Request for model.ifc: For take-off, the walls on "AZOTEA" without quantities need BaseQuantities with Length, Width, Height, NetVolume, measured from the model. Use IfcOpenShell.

First a look at what the model holds.

```python
import ifcopenshell
import ifcopenshell.util.element
import ifcopenshell.util.unit

model = ifcopenshell.open("model.ifc")
print(model.schema)
for unit_type in ("LENGTHUNIT", "AREAUNIT", "VOLUMEUNIT"):
    print(unit_type, ifcopenshell.util.unit.calculate_unit_scale(model, unit_type))
storey = next(s for s in model.by_type("IfcBuildingStorey") if s.Name == "AZOTEA")
walls = [e for e in ifcopenshell.util.element.get_decomposition(storey) if e.is_a("IfcWall")]
for e in sorted(walls, key=lambda e: e.id()):
    print(e.id(), e.is_a(), e.Name, list(ifcopenshell.util.element.get_psets(e, qtos_only=True)), sep=" | ")
```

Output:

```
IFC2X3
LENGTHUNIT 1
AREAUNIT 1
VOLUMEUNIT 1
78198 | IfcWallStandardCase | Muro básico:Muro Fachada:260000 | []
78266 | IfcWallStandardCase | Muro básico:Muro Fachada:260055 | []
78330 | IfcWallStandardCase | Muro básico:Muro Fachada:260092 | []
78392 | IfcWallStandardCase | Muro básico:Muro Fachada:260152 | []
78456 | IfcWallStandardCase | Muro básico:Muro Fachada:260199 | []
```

```python
import ifcopenshell
import ifcopenshell.api.pset
import ifcopenshell.geom
import ifcopenshell.util.element
import ifcopenshell.util.shape
import ifcopenshell.util.unit

model = ifcopenshell.open("model.ifc")
unit_scale = ifcopenshell.util.unit.calculate_unit_scale(model)
volume_scale = ifcopenshell.util.unit.calculate_unit_scale(model, "VOLUMEUNIT")
settings = ifcopenshell.geom.settings()

storey = next(s for s in model.by_type("IfcBuildingStorey") if s.Name == "AZOTEA")
walls = [e for e in ifcopenshell.util.element.get_decomposition(storey) if e.is_a("IfcWall")]

for e in sorted(walls, key=lambda e: e.id()):
    if ifcopenshell.util.element.get_psets(e, qtos_only=True, should_inherit=False):
        continue
    # Geometry comes back in metres, in the element's own axes.
    shape = ifcopenshell.geom.create_shape(settings, e)
    values = {
        "Length": ifcopenshell.util.shape.get_x(shape.geometry) / unit_scale,
        "Width": ifcopenshell.util.shape.get_y(shape.geometry) / unit_scale,
        "Height": ifcopenshell.util.shape.get_z(shape.geometry) / unit_scale,
        "NetVolume": ifcopenshell.util.shape.get_volume(shape.geometry) / volume_scale,
    }
    qto = ifcopenshell.api.pset.add_qto(model, product=e, name="BaseQuantities")
    ifcopenshell.api.pset.edit_qto(model, qto=qto, properties=values)
    print(e.id(), {k: round(v, 3) for k, v in values.items()})

model.write("model_v2.ifc")
```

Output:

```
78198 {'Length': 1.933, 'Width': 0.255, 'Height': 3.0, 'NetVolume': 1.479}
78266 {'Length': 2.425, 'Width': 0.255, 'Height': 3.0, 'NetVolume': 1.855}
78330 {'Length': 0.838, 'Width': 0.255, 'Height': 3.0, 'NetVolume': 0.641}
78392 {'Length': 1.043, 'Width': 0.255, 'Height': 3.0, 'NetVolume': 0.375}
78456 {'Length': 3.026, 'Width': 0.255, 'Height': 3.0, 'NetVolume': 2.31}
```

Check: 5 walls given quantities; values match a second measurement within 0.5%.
